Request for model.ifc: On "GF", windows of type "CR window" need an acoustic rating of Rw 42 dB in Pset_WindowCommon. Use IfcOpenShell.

First a look at what the model holds.

```python
import ifcopenshell
import ifcopenshell.util.element

model = ifcopenshell.open("model.ifc")
print(model.schema)
storey = next(s for s in model.by_type("IfcBuildingStorey") if s.Name == "GF")
windows = [e for e in ifcopenshell.util.element.get_decomposition(storey) if e.is_a("IfcWindow")]
seen = {}
for e in windows:
    element_type = ifcopenshell.util.element.get_type(e)
    key = (element_type.Name if element_type != e and element_type else None, ifcopenshell.util.element.get_pset(e, "Pset_WindowCommon", "AcousticRating"))
    seen[key] = seen.get(key, 0) + 1
for (name, value), count in sorted(seen.items(), key=str):
    print(count, "x", name, "|", value)
```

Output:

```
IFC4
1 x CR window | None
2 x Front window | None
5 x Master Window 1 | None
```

```python
import ifcopenshell
import ifcopenshell.api.pset
import ifcopenshell.util.element

model = ifcopenshell.open("model.ifc")

storey = next(s for s in model.by_type("IfcBuildingStorey") if s.Name == "GF")
windows = [e for e in ifcopenshell.util.element.get_decomposition(storey) if e.is_a("IfcWindow")]

count = 0
for e in windows:
    element_type = ifcopenshell.util.element.get_type(e)
    if element_type in (None, e) or element_type.Name != "CR window":
        continue
    # add_pset returns the element's existing set when there is one.
    pset = ifcopenshell.api.pset.add_pset(model, product=e, name="Pset_WindowCommon")
    ifcopenshell.api.pset.edit_pset(model, pset=pset, properties={"AcousticRating": "Rw 42 dB"})
    count += 1

print(count, "windows updated")

model.write("model_rev.ifc")
```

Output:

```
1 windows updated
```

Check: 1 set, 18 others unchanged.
